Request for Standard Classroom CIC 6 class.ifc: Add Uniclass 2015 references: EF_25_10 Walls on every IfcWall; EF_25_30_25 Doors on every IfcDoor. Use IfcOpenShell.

First a look at what the model holds.

```python
import ifcopenshell

model = ifcopenshell.open("Standard Classroom CIC 6 class.ifc")
print(model.schema)
print("classifications:", [c.Name for c in model.by_type("IfcClassification")])
for ifc_class in ("IfcDoor", "IfcRoof", "IfcStair", "IfcWall", "IfcWindow"):
    print(ifc_class, len(model.by_type(ifc_class)))
```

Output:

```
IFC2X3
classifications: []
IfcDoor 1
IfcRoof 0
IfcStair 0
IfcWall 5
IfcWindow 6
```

```python
import ifcopenshell
import ifcopenshell.api.classification

model = ifcopenshell.open("Standard Classroom CIC 6 class.ifc")

# IFC2X3 requires Source and Edition and has no link from the project to the system.
system = model.create_entity("IfcClassification", Source="NBS", Edition="2015", Name="Uniclass 2015")

codes = {
    "IfcWall": ("EF_25_10", "Walls"),
    "IfcDoor": ("EF_25_30_25", "Doors"),
}
for ifc_class, (code, name) in codes.items():
    products = model.by_type(ifc_class)
    ifcopenshell.api.classification.add_reference(
        model, products=products, classification=system, identification=code, name=name
    )
    print(code, len(products))

model.write("Standard Classroom CIC 6 class-out.ifc")
```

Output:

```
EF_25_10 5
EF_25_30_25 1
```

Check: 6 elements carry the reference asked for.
